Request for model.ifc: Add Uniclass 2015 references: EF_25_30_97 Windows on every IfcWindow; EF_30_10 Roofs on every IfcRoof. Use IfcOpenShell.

First a look at what the model holds.

```python
import ifcopenshell

model = ifcopenshell.open("model.ifc")
print(model.schema)
print("classifications:", [c.Name for c in model.by_type("IfcClassification")])
for ifc_class in ("IfcDoor", "IfcRoof", "IfcStair", "IfcWall", "IfcWindow"):
    print(ifc_class, len(model.by_type(ifc_class)))
```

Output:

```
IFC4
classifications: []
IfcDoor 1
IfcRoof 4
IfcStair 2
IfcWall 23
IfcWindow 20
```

```python
import ifcopenshell
import ifcopenshell.api.classification

model = ifcopenshell.open("model.ifc")

system = ifcopenshell.api.classification.add_classification(model, classification="Uniclass 2015")

codes = {
    "IfcWindow": ("EF_25_30_97", "Windows"),
    "IfcRoof": ("EF_30_10", "Roofs"),
}
for ifc_class, (code, name) in codes.items():
    products = model.by_type(ifc_class)
    ifcopenshell.api.classification.add_reference(
        model, products=products, classification=system, identification=code, name=name
    )
    print(code, len(products))

model.write("model_v2.ifc")
```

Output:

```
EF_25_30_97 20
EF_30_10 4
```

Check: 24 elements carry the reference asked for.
